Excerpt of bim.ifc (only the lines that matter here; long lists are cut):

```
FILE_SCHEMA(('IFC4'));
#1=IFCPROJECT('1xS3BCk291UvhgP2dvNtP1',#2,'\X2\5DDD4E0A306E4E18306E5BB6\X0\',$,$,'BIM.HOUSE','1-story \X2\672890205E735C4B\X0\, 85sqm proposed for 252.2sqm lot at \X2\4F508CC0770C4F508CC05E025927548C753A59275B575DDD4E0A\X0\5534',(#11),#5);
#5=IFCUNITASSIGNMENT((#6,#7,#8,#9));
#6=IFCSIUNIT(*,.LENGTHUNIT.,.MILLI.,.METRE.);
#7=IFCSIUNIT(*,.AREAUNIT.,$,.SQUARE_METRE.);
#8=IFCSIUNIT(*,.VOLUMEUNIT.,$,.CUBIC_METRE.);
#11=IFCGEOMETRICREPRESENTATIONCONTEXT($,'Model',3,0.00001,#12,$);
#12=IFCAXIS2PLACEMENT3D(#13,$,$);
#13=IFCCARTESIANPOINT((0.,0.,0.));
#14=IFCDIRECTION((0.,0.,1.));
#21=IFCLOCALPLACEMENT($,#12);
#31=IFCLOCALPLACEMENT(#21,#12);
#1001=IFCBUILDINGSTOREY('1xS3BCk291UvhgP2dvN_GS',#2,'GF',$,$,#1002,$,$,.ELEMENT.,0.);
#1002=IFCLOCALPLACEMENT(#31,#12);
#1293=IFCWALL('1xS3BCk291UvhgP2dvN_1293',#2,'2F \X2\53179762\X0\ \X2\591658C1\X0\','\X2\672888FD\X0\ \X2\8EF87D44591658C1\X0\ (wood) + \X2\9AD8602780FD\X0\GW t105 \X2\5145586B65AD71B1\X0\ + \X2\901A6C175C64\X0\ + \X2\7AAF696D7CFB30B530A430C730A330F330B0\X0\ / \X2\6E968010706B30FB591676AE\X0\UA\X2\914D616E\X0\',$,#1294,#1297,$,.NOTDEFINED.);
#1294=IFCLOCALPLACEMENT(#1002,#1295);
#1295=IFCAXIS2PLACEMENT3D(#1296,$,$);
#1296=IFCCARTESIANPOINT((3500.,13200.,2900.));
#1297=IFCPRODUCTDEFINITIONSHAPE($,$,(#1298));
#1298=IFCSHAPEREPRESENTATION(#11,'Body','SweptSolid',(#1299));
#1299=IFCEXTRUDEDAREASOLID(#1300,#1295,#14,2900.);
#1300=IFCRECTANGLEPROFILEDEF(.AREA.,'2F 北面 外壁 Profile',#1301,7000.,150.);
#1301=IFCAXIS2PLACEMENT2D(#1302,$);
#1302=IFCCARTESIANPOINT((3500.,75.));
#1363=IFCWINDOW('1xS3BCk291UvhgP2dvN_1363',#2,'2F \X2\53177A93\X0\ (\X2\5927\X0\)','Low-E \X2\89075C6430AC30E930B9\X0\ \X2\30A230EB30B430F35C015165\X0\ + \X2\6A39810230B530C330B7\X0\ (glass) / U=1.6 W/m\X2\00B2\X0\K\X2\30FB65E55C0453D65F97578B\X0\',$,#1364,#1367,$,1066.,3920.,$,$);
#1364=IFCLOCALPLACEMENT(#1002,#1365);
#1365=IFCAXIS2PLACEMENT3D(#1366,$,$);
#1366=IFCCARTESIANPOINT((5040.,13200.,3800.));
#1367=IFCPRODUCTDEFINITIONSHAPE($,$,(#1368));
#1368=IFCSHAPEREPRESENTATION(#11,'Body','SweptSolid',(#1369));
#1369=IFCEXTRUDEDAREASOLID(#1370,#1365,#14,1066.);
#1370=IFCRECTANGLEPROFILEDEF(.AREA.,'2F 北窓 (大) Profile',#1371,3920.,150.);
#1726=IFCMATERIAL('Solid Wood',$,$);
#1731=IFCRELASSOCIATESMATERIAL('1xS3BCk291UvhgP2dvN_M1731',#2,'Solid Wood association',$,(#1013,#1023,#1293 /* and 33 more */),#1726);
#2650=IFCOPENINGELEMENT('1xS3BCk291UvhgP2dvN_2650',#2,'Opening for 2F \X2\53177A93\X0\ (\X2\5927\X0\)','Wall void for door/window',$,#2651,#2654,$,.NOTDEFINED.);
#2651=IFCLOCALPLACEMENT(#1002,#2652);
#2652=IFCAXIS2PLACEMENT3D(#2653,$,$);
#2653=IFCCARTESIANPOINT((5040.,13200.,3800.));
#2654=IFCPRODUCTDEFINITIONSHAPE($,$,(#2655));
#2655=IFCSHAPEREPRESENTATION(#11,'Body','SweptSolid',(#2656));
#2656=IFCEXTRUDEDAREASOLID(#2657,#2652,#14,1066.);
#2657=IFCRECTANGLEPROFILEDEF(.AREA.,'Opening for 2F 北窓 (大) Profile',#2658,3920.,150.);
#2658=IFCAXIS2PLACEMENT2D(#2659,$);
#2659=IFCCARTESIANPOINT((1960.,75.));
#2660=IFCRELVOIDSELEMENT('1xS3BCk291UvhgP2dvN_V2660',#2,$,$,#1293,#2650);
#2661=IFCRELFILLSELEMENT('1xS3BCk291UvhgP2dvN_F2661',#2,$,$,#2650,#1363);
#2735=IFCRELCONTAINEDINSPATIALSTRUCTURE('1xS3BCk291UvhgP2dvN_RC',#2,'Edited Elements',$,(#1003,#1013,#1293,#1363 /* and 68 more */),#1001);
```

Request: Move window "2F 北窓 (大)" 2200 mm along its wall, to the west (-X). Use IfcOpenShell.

```python
import ifcopenshell
import ifcopenshell.api.geometry
import ifcopenshell.util.placement
import ifcopenshell.util.unit

model = ifcopenshell.open("bim.ifc")
unit_scale = ifcopenshell.util.unit.calculate_unit_scale(model)

window = model.by_guid("1xS3BCk291UvhgP2dvN_1363")
opening = window.FillsVoids[0].RelatingOpeningElement
wall = opening.VoidsElements[0].RelatingBuildingElement

wall_matrix = ifcopenshell.util.placement.get_local_placement(wall.ObjectPlacement)
shift = wall_matrix[:3, 0] * -2.2 / unit_scale
before = ifcopenshell.util.placement.get_local_placement(window.ObjectPlacement)[:3, 3].copy()

# The window is not placed relative to its opening, so move both.
for product in (opening, window):
    matrix = ifcopenshell.util.placement.get_local_placement(product.ObjectPlacement)
    matrix[:3, 3] += shift
    ifcopenshell.api.geometry.edit_object_placement(model, product=product, matrix=matrix, is_si=False)

after = ifcopenshell.util.placement.get_local_placement(window.ObjectPlacement)[:3, 3]
print("window moved by", (after - before).round(3) + 0.0)

model.write("bim_edited.ifc")
```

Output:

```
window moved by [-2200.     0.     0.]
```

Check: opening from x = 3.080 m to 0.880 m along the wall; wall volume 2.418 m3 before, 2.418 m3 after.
